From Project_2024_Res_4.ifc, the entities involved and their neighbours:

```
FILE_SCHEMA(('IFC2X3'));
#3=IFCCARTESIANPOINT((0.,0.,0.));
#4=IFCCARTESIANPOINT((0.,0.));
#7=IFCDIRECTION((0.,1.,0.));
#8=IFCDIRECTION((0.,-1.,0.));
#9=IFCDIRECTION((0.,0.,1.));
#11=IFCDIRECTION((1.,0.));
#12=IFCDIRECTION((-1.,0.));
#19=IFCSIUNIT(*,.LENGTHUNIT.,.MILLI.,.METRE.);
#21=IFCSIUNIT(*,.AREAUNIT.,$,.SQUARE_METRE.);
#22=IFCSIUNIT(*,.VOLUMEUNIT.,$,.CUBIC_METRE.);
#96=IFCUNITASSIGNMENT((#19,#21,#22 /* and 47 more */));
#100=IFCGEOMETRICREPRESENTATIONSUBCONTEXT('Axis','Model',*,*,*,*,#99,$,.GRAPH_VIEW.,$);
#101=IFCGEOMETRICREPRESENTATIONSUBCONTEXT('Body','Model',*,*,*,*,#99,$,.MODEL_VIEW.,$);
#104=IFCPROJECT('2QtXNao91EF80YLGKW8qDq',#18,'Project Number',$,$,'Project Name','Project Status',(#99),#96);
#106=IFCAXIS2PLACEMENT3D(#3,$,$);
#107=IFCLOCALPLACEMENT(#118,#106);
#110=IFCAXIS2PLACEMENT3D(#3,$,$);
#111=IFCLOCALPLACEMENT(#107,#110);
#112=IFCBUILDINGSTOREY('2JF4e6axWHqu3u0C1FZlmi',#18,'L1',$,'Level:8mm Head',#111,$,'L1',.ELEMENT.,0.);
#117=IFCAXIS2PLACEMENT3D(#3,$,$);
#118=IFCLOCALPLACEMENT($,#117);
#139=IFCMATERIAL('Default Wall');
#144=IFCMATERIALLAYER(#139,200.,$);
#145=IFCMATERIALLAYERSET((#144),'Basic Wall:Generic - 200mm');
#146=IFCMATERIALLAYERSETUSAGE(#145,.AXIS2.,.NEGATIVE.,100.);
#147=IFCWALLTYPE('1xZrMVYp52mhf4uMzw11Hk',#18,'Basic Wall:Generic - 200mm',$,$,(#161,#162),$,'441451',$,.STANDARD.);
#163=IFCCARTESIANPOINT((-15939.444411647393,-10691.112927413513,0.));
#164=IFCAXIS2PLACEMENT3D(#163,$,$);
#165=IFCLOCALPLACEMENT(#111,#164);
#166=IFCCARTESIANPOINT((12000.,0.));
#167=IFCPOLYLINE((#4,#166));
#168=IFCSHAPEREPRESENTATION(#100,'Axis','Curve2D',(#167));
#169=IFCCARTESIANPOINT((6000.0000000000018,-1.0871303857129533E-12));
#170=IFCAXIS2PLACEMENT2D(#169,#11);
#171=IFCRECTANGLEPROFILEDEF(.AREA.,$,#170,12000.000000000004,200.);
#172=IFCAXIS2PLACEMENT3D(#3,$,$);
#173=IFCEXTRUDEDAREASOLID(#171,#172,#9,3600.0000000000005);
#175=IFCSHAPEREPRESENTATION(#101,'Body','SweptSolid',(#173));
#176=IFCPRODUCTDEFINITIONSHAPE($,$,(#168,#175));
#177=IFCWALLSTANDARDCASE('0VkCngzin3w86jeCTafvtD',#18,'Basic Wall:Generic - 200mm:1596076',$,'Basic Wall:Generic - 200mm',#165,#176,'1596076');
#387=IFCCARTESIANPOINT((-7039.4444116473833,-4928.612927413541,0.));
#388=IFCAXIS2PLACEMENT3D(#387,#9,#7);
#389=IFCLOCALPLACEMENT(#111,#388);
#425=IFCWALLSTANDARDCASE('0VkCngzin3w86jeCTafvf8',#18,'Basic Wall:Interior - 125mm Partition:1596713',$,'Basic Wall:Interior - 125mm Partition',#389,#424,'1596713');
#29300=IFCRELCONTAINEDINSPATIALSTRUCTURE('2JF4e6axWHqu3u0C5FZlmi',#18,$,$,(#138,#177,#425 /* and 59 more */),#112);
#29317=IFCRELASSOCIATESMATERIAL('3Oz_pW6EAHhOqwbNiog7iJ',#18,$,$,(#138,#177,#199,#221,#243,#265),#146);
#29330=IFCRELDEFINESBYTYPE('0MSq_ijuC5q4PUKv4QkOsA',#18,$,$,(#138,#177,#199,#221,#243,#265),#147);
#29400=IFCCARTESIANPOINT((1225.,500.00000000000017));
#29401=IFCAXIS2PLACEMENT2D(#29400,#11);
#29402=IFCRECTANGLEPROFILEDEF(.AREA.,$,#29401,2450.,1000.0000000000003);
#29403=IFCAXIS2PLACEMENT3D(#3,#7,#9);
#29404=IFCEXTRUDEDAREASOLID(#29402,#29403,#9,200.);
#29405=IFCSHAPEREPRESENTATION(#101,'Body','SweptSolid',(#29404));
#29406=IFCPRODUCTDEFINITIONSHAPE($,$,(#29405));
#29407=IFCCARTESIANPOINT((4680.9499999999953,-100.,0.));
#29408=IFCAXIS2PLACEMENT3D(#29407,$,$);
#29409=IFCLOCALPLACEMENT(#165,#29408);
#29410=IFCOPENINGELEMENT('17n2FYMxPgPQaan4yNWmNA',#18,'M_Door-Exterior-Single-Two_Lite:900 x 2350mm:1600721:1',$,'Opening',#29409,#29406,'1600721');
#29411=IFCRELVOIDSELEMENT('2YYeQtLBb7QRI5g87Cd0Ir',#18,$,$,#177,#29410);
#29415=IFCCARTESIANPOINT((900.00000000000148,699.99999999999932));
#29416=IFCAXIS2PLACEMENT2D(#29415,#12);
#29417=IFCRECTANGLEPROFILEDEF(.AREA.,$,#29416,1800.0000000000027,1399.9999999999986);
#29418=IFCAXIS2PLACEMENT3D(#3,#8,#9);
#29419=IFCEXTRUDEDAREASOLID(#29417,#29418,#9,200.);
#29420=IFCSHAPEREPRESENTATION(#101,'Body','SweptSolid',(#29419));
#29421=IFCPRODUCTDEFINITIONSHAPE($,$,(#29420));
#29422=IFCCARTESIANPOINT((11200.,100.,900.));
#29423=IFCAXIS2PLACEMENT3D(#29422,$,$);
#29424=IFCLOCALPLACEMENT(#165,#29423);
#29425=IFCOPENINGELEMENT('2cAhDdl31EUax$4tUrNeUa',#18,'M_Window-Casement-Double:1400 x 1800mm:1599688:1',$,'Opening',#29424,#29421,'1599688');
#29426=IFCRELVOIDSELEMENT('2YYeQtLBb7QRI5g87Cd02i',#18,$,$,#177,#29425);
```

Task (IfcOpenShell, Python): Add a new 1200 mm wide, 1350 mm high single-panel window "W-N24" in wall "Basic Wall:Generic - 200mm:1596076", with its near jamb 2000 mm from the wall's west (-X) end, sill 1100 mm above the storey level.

```python
import numpy as np
import ifcopenshell
import ifcopenshell.api.feature
import ifcopenshell.api.geometry
import ifcopenshell.api.root
import ifcopenshell.api.spatial
import ifcopenshell.api.type
import ifcopenshell.geom
import ifcopenshell.util.element
import ifcopenshell.util.placement
import ifcopenshell.util.representation
import ifcopenshell.util.shape
import ifcopenshell.util.unit

model = ifcopenshell.open("Project_2024_Res_4.ifc")
unit_scale = ifcopenshell.util.unit.calculate_unit_scale(model)
settings = ifcopenshell.geom.settings()


def volume(element):
    """Net volume in cubic metres, openings subtracted."""
    shape = ifcopenshell.geom.create_shape(settings, element)
    return ifcopenshell.util.shape.get_volume(shape.geometry)


wall = model.by_guid("0VkCngzin3w86jeCTafvtD")
storey = ifcopenshell.util.element.get_container(wall, ifc_class="IfcBuildingStorey")
context = ifcopenshell.util.representation.get_context(model, "Model", "Body", "MODEL_VIEW")
before = volume(wall)

width, height, from_end, sill = 1.2, 1.35, 2, 1.1  # metres

# The wall runs along its own X axis, and the end named is its -X end.
wall_shape = ifcopenshell.geom.create_shape(settings, wall)
x, y, z = ifcopenshell.util.shape.get_vertices(wall_shape.geometry).T
start = x.min() + from_end
face, thickness = float(y.min()), float(y.max() - y.min())
wall_matrix = ifcopenshell.util.placement.get_local_placement(wall.ObjectPlacement)
level = ifcopenshell.util.placement.get_local_placement(storey.ObjectPlacement)[2, 3]


def in_wall(x, y):
    """Placement at x, y metres in the wall's axes, at sill height."""
    matrix = wall_matrix.copy()
    matrix[:, 3] = wall_matrix @ np.array([x / unit_scale, y / unit_scale, 0.0, 1.0])
    matrix[2, 3] = level + sill / unit_scale
    return matrix


# Opening: a box that overshoots both wall faces by 50 mm.
opening = ifcopenshell.api.root.create_entity(model, ifc_class="IfcOpeningElement")
box = ifcopenshell.api.geometry.add_wall_representation(
    model, context=context, length=width, height=height, thickness=thickness + 0.1
)
ifcopenshell.api.geometry.assign_representation(model, product=opening, representation=box)
ifcopenshell.api.geometry.edit_object_placement(model, product=opening, matrix=in_wall(start, face - 0.05), is_si=False)
ifcopenshell.api.feature.add_feature(model, feature=opening, element=wall)

window = ifcopenshell.api.root.create_entity(model, ifc_class="IfcWindow", name="W-N24")
window.OverallWidth, window.OverallHeight = width / unit_scale, height / unit_scale
body = ifcopenshell.api.geometry.add_window_representation(
    model,
    context=context,
    overall_width=window.OverallWidth,
    overall_height=window.OverallHeight,
    partition_type="SINGLE_PANEL",
)
ifcopenshell.api.geometry.assign_representation(model, product=window, representation=body)
ifcopenshell.api.spatial.assign_container(model, products=[window], relating_structure=storey)
fills = ifcopenshell.api.feature.add_filling(model, opening=opening, element=window)
fills.OwnerHistory = window.OwnerHistory  # required in IFC2X3

# IFC2X3 keeps the operation on the window style.
style = ifcopenshell.api.root.create_entity(model, ifc_class="IfcWindowStyle", name="W-N24")
style.OperationType, style.ConstructionType = "SINGLE_PANEL", "NOTDEFINED"
style.ParameterTakesPrecedence = style.Sizeable = False
ifcopenshell.api.type.assign_type(model, related_objects=[window], relating_type=style)

# Centre the window in the wall's thickness.
ifcopenshell.api.geometry.edit_object_placement(model, product=window, matrix=in_wall(start, face), is_si=False)
window_shape = ifcopenshell.geom.create_shape(settings, window)
depth = ifcopenshell.util.shape.get_vertices(window_shape.geometry)[:, 1]
offset = face + thickness / 2 - (depth.min() + depth.max()) / 2
ifcopenshell.api.geometry.edit_object_placement(model, product=window, matrix=in_wall(start, offset), is_si=False)

after = volume(wall)

print(f"wall volume {before:.3f} -> {after:.3f} m3")

model.write("Project_2024_Res_4_updated.ifc")
```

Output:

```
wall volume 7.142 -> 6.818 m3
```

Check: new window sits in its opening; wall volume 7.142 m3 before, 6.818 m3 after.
